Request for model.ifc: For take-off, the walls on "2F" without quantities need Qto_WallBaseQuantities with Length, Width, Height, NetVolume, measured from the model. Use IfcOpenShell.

First a look at what the model holds.

```python
import ifcopenshell
import ifcopenshell.util.element
import ifcopenshell.util.unit

model = ifcopenshell.open("model.ifc")
print(model.schema)
for unit_type in ("LENGTHUNIT", "AREAUNIT", "VOLUMEUNIT"):
    print(unit_type, ifcopenshell.util.unit.calculate_unit_scale(model, unit_type))
storey = next(s for s in model.by_type("IfcBuildingStorey") if s.Name == "2F")
walls = [e for e in ifcopenshell.util.element.get_decomposition(storey) if e.is_a("IfcWall")]
for e in sorted(walls, key=lambda e: e.id()):
    print(e.id(), e.is_a(), e.Name, list(ifcopenshell.util.element.get_psets(e, qtos_only=True)), sep=" | ")
```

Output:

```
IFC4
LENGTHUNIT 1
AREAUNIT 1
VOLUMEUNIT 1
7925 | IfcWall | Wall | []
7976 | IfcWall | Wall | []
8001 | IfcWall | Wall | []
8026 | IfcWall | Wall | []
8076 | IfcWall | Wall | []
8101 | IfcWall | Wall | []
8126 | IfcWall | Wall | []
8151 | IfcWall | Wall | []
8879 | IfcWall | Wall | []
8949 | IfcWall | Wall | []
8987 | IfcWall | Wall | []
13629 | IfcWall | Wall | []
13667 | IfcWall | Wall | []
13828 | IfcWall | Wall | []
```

```python
import ifcopenshell
import ifcopenshell.api.pset
import ifcopenshell.geom
import ifcopenshell.util.element
import ifcopenshell.util.shape
import ifcopenshell.util.unit

model = ifcopenshell.open("model.ifc")
unit_scale = ifcopenshell.util.unit.calculate_unit_scale(model)
volume_scale = ifcopenshell.util.unit.calculate_unit_scale(model, "VOLUMEUNIT")
settings = ifcopenshell.geom.settings()

storey = next(s for s in model.by_type("IfcBuildingStorey") if s.Name == "2F")
walls = [e for e in ifcopenshell.util.element.get_decomposition(storey) if e.is_a("IfcWall")]

for e in sorted(walls, key=lambda e: e.id()):
    if ifcopenshell.util.element.get_psets(e, qtos_only=True, should_inherit=False):
        continue
    # Geometry comes back in metres, in the element's own axes.
    shape = ifcopenshell.geom.create_shape(settings, e)
    values = {
        "Length": ifcopenshell.util.shape.get_x(shape.geometry) / unit_scale,
        "Width": ifcopenshell.util.shape.get_y(shape.geometry) / unit_scale,
        "Height": ifcopenshell.util.shape.get_z(shape.geometry) / unit_scale,
        "NetVolume": ifcopenshell.util.shape.get_volume(shape.geometry) / volume_scale,
    }
    qto = ifcopenshell.api.pset.add_qto(model, product=e, name="Qto_WallBaseQuantities")
    ifcopenshell.api.pset.edit_qto(model, qto=qto, properties=values)
    print(e.id(), {k: round(v, 3) for k, v in values.items()})

model.write("model_v2.ifc")
```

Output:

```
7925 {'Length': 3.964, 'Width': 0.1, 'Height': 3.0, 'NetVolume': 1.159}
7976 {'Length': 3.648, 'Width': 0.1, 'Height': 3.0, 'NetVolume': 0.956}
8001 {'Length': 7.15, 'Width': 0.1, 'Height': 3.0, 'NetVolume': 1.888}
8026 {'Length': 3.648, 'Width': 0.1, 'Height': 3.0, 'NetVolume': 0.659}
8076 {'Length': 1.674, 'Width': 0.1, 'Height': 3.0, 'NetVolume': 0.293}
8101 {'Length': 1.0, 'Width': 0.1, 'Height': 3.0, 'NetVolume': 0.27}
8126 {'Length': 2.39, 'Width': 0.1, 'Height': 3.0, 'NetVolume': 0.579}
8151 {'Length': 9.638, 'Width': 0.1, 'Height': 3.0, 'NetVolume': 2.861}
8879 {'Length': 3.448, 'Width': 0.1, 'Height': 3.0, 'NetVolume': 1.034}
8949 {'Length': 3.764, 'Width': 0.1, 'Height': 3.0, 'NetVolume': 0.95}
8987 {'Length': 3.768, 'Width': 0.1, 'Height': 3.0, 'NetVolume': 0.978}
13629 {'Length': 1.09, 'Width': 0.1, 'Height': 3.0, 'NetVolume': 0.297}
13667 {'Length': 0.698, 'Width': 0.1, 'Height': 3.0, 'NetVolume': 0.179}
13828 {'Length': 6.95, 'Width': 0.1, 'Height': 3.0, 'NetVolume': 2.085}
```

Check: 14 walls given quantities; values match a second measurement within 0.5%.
